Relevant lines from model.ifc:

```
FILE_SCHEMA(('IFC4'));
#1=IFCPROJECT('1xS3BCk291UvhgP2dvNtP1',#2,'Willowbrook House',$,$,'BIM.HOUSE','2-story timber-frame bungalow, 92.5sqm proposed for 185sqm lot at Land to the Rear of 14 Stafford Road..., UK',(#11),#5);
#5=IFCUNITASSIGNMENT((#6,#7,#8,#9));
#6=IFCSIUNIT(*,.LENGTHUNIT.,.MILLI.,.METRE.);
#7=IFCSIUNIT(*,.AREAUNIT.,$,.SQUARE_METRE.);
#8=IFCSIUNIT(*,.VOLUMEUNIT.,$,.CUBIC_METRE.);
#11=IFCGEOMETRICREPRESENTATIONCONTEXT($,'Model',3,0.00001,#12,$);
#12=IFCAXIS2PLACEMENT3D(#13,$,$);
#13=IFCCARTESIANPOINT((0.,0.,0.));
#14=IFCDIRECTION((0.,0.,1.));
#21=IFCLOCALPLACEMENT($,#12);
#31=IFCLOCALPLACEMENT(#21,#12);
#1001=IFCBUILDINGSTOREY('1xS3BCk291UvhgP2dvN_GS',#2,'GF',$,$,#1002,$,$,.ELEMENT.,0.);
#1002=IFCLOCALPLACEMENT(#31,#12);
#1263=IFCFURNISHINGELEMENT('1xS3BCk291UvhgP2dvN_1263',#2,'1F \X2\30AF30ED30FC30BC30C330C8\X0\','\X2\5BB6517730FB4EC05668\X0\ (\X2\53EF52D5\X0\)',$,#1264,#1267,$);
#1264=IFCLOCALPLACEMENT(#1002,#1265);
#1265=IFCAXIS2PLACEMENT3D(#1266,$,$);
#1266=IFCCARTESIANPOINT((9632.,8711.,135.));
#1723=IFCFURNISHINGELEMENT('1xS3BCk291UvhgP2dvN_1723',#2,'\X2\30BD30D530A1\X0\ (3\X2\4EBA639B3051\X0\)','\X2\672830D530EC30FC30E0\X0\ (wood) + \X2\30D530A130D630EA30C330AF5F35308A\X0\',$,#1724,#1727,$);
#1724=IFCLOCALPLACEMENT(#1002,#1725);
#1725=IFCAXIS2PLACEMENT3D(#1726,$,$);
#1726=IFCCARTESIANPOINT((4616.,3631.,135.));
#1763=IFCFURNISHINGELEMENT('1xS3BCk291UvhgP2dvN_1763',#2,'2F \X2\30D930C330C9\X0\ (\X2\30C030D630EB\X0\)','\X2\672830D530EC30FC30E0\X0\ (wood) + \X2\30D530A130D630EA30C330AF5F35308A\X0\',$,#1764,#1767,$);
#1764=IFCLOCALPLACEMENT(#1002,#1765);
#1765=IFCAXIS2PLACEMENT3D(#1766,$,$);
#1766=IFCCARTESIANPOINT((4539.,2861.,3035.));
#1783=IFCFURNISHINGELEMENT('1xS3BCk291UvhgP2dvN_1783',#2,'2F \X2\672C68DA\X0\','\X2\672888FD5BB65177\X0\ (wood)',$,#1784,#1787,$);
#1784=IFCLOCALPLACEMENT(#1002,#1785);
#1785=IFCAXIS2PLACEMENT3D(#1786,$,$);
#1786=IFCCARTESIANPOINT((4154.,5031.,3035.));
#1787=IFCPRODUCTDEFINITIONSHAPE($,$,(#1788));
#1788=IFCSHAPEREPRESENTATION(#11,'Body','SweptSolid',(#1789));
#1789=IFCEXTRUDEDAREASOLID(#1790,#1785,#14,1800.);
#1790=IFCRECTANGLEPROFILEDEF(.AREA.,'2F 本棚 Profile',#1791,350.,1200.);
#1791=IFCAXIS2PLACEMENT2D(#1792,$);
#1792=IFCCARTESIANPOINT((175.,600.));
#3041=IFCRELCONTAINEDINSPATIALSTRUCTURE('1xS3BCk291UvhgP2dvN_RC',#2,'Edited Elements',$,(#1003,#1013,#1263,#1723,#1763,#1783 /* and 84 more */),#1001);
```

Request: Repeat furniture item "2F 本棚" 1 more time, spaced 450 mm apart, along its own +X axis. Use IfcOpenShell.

```python
import ifcopenshell
import ifcopenshell.api.geometry
import ifcopenshell.api.root
import ifcopenshell.util.element
import ifcopenshell.util.placement
import ifcopenshell.util.unit

model = ifcopenshell.open("model.ifc")
unit_scale = ifcopenshell.util.unit.calculate_unit_scale(model)


def reuse_history(source, copy):
    """copy_class also copies each property set's owner history, people and application; keep the originals."""
    for rel in copy.IsDefinedBy:
        if rel.is_a("IfcRelDefinesByProperties") and (history := rel.RelatingPropertyDefinition.OwnerHistory):
            rel.RelatingPropertyDefinition.OwnerHistory = source.OwnerHistory
            ifcopenshell.util.element.remove_deep2(model, history)


source = model.by_id(1783)
base = ifcopenshell.util.placement.get_local_placement(source.ObjectPlacement)
step = base[:3, 0] * 0.45 / unit_scale

for i in range(1, 2):
    copy = ifcopenshell.api.root.copy_class(model, product=source)
    copy.Representation = ifcopenshell.util.element.copy_deep(
        model, source.Representation, exclude=["IfcGeometricRepresentationContext", "IfcRepresentationMap"]
    )
    reuse_history(source, copy)
    matrix = base.copy()
    matrix[:3, 3] += i * step
    print("added at", matrix[:3, 3].round(3) + 0.0)
    ifcopenshell.api.geometry.edit_object_placement(model, product=copy, matrix=matrix, is_si=False)

model.write("model_v2.ifc")
```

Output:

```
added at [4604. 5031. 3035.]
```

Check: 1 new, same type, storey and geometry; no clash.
